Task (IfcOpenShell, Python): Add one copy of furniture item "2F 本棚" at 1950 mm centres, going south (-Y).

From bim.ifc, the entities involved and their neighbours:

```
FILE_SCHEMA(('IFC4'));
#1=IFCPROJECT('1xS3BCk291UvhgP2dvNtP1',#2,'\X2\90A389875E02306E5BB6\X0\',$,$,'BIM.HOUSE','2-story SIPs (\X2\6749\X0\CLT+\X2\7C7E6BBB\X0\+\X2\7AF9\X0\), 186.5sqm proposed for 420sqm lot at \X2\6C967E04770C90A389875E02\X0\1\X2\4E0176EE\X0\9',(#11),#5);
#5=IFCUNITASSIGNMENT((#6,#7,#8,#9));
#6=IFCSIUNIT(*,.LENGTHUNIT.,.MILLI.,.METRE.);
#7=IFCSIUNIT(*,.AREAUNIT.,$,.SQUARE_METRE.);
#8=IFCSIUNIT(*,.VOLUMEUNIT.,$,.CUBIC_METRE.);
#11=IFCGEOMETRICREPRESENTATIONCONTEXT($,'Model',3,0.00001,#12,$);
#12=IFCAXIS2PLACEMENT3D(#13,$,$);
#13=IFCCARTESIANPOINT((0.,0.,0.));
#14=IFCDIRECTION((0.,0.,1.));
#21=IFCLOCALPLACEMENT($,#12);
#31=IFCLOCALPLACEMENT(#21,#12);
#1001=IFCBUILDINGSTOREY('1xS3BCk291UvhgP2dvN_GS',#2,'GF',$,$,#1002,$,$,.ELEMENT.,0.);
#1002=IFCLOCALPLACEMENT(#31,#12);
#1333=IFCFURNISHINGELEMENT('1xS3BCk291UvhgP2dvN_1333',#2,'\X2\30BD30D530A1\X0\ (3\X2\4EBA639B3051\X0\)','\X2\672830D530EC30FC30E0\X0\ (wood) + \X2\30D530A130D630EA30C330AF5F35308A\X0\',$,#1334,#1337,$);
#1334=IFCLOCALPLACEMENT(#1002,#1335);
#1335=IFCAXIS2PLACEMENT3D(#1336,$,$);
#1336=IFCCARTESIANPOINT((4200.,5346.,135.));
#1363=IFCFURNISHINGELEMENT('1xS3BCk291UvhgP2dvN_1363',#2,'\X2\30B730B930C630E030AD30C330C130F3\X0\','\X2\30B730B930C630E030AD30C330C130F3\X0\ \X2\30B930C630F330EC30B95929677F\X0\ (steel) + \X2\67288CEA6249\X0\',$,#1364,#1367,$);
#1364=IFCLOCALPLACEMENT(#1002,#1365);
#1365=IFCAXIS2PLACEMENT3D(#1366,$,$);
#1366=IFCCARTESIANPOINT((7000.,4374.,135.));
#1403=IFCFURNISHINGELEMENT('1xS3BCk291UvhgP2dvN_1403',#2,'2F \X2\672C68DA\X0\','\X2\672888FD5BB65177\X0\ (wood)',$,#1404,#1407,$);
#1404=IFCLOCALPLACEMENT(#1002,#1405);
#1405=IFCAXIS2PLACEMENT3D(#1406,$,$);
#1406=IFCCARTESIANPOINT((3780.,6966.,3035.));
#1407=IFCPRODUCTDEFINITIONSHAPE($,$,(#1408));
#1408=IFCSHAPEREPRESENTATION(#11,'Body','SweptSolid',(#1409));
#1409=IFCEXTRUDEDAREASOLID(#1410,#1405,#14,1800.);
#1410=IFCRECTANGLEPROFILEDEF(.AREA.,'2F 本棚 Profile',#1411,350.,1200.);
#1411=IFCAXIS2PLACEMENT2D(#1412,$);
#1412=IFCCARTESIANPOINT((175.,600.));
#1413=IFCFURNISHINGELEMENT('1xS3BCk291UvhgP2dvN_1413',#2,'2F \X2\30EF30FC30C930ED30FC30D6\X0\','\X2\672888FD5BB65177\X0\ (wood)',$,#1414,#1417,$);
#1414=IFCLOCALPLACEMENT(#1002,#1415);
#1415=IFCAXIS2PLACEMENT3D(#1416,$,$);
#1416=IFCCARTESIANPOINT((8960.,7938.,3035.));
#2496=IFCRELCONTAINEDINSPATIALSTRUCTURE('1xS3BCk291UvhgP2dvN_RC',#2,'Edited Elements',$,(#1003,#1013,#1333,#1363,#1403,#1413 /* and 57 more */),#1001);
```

```python
import numpy as np
import ifcopenshell
import ifcopenshell.api.geometry
import ifcopenshell.api.root
import ifcopenshell.util.element
import ifcopenshell.util.placement

model = ifcopenshell.open("bim.ifc")


def reuse_history(source, copy):
    """copy_class also copies each property set's owner history, people and application; keep the originals."""
    for rel in copy.IsDefinedBy:
        if rel.is_a("IfcRelDefinesByProperties") and (history := rel.RelatingPropertyDefinition.OwnerHistory):
            rel.RelatingPropertyDefinition.OwnerHistory = source.OwnerHistory
            ifcopenshell.util.element.remove_deep2(model, history)


source = model.by_id(1403)
base = ifcopenshell.util.placement.get_local_placement(source.ObjectPlacement)
step = np.array([0.0, -1.0, 0.0]) * 1950.0

for i in range(1, 2):
    copy = ifcopenshell.api.root.copy_class(model, product=source)
    copy.Representation = ifcopenshell.util.element.copy_deep(
        model, source.Representation, exclude=["IfcGeometricRepresentationContext", "IfcRepresentationMap"]
    )
    reuse_history(source, copy)
    matrix = base.copy()
    matrix[:3, 3] += i * step
    print("added at", matrix[:3, 3].round(3) + 0.0)
    ifcopenshell.api.geometry.edit_object_placement(model, product=copy, matrix=matrix, is_si=False)

model.write("bim_updated.ifc")
```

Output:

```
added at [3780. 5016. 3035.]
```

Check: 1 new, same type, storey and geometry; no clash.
